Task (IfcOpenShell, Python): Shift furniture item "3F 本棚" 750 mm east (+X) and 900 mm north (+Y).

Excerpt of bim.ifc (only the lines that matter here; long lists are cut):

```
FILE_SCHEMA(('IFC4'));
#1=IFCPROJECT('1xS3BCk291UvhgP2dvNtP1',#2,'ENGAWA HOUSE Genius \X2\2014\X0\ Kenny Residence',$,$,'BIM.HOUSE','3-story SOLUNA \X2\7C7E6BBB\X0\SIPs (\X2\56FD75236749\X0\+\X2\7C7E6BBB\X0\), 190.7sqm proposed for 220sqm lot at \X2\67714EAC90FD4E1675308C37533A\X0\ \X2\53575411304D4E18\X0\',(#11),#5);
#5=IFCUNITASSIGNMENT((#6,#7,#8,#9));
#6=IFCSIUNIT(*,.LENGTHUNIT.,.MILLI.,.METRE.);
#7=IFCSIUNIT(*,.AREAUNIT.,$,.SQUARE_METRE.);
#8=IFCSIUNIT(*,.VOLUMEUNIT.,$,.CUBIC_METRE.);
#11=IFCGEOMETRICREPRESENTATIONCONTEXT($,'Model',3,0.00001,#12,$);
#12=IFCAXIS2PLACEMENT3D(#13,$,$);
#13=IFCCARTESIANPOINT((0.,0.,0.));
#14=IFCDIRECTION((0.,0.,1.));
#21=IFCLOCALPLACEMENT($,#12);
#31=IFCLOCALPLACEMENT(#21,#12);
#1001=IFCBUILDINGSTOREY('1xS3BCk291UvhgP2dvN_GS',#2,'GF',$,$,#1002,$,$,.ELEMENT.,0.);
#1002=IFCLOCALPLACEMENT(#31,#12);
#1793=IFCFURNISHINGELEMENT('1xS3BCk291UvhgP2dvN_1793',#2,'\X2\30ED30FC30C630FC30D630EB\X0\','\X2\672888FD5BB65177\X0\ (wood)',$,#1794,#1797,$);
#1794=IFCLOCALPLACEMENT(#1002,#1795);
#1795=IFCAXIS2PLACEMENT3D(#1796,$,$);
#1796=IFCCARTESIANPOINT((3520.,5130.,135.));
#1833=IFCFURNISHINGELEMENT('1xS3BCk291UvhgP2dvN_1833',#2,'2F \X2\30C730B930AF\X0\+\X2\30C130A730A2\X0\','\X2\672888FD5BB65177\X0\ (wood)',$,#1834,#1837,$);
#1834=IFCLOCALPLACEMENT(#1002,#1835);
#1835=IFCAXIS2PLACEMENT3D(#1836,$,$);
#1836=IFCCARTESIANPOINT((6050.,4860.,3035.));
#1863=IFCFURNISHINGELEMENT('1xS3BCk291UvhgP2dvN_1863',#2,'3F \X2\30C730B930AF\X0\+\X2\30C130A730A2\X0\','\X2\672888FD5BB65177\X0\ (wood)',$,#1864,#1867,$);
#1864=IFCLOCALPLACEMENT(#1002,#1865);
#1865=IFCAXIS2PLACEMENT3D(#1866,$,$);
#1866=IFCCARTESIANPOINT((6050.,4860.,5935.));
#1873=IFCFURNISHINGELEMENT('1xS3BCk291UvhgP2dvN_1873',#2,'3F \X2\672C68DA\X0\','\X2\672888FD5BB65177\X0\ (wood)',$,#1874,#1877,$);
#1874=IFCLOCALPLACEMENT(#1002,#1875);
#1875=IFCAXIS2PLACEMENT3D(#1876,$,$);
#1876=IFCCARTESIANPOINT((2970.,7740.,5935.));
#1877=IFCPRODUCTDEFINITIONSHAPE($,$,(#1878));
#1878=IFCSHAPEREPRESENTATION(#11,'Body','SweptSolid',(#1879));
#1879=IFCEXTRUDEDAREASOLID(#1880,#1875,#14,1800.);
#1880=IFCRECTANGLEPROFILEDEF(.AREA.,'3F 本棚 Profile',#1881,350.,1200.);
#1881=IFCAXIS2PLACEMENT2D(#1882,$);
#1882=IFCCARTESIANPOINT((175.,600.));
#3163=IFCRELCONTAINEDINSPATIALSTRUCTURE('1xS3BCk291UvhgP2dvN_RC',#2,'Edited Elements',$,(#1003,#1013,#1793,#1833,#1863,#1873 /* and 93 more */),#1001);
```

```python
import ifcopenshell
import ifcopenshell.api.geometry
import ifcopenshell.util.placement
import ifcopenshell.util.unit

model = ifcopenshell.open("bim.ifc")
unit_scale = ifcopenshell.util.unit.calculate_unit_scale(model)

item = model.by_guid("1xS3BCk291UvhgP2dvN_1873")
matrix = ifcopenshell.util.placement.get_local_placement(item.ObjectPlacement)
matrix[0, 3] += 0.75 / unit_scale
matrix[1, 3] += 0.9 / unit_scale
ifcopenshell.api.geometry.edit_object_placement(model, product=item, matrix=matrix, is_si=False)

print(ifcopenshell.util.placement.get_local_placement(item.ObjectPlacement).round(3) + 0.0)

model.write("bim_rev.ifc")
```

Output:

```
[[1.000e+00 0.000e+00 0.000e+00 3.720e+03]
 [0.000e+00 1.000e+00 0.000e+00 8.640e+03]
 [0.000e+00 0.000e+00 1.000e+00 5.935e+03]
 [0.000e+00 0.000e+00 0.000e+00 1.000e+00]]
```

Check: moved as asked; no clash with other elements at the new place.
